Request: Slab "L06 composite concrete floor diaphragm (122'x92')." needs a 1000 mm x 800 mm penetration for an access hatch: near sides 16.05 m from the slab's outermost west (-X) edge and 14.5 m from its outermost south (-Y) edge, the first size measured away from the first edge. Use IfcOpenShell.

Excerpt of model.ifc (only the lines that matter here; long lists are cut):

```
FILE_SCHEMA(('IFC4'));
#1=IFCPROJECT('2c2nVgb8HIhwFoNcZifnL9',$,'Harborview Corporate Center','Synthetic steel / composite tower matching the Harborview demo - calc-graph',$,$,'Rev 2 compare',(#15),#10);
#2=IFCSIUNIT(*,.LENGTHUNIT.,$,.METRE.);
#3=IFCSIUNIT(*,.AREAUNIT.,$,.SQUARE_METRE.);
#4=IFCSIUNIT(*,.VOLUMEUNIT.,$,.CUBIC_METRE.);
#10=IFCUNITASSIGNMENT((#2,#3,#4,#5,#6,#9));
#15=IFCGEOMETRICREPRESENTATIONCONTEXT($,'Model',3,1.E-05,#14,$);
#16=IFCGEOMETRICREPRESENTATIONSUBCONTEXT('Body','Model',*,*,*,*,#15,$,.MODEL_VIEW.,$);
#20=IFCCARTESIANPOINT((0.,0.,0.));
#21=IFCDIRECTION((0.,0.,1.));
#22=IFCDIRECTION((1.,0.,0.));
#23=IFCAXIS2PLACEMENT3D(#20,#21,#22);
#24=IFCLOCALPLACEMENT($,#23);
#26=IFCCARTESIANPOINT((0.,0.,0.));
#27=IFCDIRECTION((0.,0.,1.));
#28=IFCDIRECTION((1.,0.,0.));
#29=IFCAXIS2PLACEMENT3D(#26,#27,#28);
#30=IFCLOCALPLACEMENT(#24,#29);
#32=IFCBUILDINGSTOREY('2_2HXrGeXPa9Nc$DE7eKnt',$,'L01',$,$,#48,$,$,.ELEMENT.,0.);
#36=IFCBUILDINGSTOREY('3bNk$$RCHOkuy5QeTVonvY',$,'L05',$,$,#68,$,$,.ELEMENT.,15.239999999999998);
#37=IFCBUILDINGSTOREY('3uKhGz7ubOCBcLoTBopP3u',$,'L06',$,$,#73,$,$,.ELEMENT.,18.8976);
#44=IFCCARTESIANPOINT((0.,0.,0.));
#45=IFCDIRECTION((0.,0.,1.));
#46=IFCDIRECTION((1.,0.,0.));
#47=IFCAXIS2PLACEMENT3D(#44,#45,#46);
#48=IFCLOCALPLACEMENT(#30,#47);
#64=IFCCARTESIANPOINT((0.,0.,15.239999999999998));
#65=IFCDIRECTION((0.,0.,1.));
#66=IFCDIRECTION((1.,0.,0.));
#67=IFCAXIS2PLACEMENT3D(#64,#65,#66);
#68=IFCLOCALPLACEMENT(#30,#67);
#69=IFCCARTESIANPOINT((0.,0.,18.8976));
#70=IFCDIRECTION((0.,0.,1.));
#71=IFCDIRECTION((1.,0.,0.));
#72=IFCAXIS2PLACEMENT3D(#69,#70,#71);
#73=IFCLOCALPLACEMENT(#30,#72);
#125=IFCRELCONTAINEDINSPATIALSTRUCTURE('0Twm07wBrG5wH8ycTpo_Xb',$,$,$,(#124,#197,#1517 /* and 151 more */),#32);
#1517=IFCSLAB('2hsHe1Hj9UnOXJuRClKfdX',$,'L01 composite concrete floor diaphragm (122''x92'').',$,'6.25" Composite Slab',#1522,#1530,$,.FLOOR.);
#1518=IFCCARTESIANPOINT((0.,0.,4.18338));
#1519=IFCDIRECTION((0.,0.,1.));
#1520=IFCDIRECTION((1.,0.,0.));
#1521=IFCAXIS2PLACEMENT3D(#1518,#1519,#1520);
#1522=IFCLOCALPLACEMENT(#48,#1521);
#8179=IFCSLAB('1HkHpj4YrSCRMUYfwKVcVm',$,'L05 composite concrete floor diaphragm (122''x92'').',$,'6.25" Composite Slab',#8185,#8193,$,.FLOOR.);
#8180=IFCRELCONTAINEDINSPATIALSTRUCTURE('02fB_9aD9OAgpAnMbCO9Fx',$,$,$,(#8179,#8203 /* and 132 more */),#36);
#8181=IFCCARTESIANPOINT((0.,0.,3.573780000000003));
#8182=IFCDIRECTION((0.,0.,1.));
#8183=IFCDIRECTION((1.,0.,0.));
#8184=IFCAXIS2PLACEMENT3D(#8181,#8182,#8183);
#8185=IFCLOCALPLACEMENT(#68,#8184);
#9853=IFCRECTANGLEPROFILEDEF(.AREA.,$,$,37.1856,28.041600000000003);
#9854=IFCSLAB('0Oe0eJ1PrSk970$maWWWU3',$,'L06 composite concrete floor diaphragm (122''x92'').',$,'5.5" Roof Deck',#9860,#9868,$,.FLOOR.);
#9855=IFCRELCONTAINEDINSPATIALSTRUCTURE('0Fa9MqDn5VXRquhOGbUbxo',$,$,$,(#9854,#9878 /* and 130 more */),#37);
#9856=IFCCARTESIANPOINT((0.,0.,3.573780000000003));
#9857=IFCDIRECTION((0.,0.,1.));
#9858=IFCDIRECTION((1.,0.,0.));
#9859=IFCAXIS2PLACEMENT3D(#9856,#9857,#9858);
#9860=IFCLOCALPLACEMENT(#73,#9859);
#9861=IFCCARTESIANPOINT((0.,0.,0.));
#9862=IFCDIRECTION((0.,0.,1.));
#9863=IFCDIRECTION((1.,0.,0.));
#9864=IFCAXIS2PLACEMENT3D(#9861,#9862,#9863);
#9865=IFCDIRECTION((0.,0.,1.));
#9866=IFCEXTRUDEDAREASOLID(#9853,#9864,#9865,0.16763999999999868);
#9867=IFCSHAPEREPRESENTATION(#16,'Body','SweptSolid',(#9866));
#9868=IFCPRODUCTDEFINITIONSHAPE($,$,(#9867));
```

```python
import numpy as np
import ifcopenshell
import ifcopenshell.api.feature
import ifcopenshell.api.geometry
import ifcopenshell.api.root
import ifcopenshell.geom
import ifcopenshell.util.placement
import ifcopenshell.util.representation
import ifcopenshell.util.shape
import ifcopenshell.util.unit

model = ifcopenshell.open("model.ifc")
unit_scale = ifcopenshell.util.unit.calculate_unit_scale(model)
settings = ifcopenshell.geom.settings()


def volume(element):
    """Net volume in cubic metres, openings subtracted."""
    shape = ifcopenshell.geom.create_shape(settings, element)
    return ifcopenshell.util.shape.get_volume(shape.geometry)


slab = model.by_guid("0Oe0eJ1PrSk970$maWWWU3")
before = volume(slab)

# Extent in the slab's own axes, in metres. The edges named are its -X and -Y sides.
slab_shape = ifcopenshell.geom.create_shape(settings, slab)
vertices = ifcopenshell.util.shape.get_vertices(slab_shape.geometry)
x_min, y_min, bottom = vertices.min(axis=0)
top = vertices[:, 2].max()

opening = ifcopenshell.api.root.create_entity(model, ifc_class="IfcOpeningElement", name="Access hatch opening", predefined_type="OPENING")
context = ifcopenshell.util.representation.get_context(model, "Model", "Body", "MODEL_VIEW")
width, depth = 1, 0.8
outline = [(0.0, 0.0), (width, 0.0), (width, depth), (0.0, depth), (0.0, 0.0)]
# Overshoot both faces by 50 mm so the cut is clean.
shape = ifcopenshell.api.geometry.add_slab_representation(
    model, context=context, depth=top - bottom + 0.1, polyline=outline
)
ifcopenshell.api.geometry.assign_representation(model, product=opening, representation=shape)

matrix = ifcopenshell.util.placement.get_local_placement(slab.ObjectPlacement)
matrix[:, 3] = matrix @ np.append(np.array([x_min + 16.05, y_min + 14.5, bottom - 0.05]) / unit_scale, 1.0)
ifcopenshell.api.geometry.edit_object_placement(model, product=opening, matrix=matrix, is_si=False)
ifcopenshell.api.feature.add_feature(model, feature=opening, element=slab)

after = volume(slab)

print(f"slab volume {before:.3f} -> {after:.3f} m3")

model.write("model_updated.ifc")
```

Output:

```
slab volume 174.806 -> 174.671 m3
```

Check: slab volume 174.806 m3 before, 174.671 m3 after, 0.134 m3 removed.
